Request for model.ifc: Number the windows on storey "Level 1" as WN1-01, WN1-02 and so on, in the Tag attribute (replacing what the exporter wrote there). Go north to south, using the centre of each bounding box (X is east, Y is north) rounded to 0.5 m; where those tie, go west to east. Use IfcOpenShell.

First a look at what the model holds.

```python
import ifcopenshell
import ifcopenshell.util.element
import ifcopenshell.util.placement

model = ifcopenshell.open("model.ifc")
print(model.schema)
storey = next(s for s in model.by_type("IfcBuildingStorey") if s.Name == "Level 1")
windows = [e for e in ifcopenshell.util.element.get_decomposition(storey) if e.is_a("IfcWindow")]
for e in sorted(windows, key=lambda e: e.id()):
    origin = ifcopenshell.util.placement.get_local_placement(e.ObjectPlacement)[:3, 3]
    print(e.id(), e.Tag, e.Name, origin.round(2) + 0.0, sep=" | ")
```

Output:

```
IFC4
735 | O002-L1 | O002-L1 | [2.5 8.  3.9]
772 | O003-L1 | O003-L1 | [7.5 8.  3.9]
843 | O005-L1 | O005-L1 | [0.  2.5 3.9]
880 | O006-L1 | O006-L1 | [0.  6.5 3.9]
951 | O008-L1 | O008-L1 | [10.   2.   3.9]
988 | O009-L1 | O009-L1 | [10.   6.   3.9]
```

```python
import ifcopenshell
import ifcopenshell.geom
import ifcopenshell.util.element
import ifcopenshell.util.shape

model = ifcopenshell.open("model.ifc")
settings = ifcopenshell.geom.settings()
settings.set("use-world-coords", True)


def centre(element):
    shape = ifcopenshell.geom.create_shape(settings, element)
    return ifcopenshell.util.shape.get_bbox_centroid(shape.geometry)


storey = next(s for s in model.by_type("IfcBuildingStorey") if s.Name == "Level 1")
windows = [e for e in ifcopenshell.util.element.get_decomposition(storey) if e.is_a("IfcWindow")]

# Insertion points can sit at a corner or the storey origin, so sort by the geometry (in metres).
centres = {e: centre(e) for e in windows}
windows.sort(key=lambda e: (-round(centres[e][1] / 0.5), centres[e][0]))

for i, e in enumerate(windows, start=1):
    number = f"WN1-{i:02d}"
    e.Tag = number
    print(e.id(), number)

model.write("model_rev.ifc")
```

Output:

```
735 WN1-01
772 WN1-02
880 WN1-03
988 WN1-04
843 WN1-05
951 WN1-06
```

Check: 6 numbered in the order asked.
